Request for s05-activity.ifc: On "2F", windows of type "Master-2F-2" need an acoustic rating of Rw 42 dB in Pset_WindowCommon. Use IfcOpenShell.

First a look at what the model holds.

```python
import ifcopenshell
import ifcopenshell.util.element

model = ifcopenshell.open("s05-activity.ifc")
print(model.schema)
storey = next(s for s in model.by_type("IfcBuildingStorey") if s.Name == "2F")
windows = [e for e in ifcopenshell.util.element.get_decomposition(storey) if e.is_a("IfcWindow")]
seen = {}
for e in windows:
    element_type = ifcopenshell.util.element.get_type(e)
    key = (element_type.Name if element_type != e and element_type else None, ifcopenshell.util.element.get_pset(e, "Pset_WindowCommon", "AcousticRating"))
    seen[key] = seen.get(key, 0) + 1
for (name, value), count in sorted(seen.items(), key=str):
    print(count, "x", name, "|", value)
```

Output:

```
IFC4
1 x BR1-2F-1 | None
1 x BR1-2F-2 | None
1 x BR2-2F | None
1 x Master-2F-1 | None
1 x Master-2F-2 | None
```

```python
import ifcopenshell
import ifcopenshell.api.pset
import ifcopenshell.util.element

model = ifcopenshell.open("s05-activity.ifc")

storey = next(s for s in model.by_type("IfcBuildingStorey") if s.Name == "2F")
windows = [e for e in ifcopenshell.util.element.get_decomposition(storey) if e.is_a("IfcWindow")]

count = 0
for e in windows:
    element_type = ifcopenshell.util.element.get_type(e)
    if element_type in (None, e) or element_type.Name != "Master-2F-2":
        continue
    # add_pset returns the element's existing set when there is one.
    pset = ifcopenshell.api.pset.add_pset(model, product=e, name="Pset_WindowCommon")
    ifcopenshell.api.pset.edit_pset(model, pset=pset, properties={"AcousticRating": "Rw 42 dB"})
    count += 1

print(count, "windows updated")

model.write("s05-activity_updated.ifc")
```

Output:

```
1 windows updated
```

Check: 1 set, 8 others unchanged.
